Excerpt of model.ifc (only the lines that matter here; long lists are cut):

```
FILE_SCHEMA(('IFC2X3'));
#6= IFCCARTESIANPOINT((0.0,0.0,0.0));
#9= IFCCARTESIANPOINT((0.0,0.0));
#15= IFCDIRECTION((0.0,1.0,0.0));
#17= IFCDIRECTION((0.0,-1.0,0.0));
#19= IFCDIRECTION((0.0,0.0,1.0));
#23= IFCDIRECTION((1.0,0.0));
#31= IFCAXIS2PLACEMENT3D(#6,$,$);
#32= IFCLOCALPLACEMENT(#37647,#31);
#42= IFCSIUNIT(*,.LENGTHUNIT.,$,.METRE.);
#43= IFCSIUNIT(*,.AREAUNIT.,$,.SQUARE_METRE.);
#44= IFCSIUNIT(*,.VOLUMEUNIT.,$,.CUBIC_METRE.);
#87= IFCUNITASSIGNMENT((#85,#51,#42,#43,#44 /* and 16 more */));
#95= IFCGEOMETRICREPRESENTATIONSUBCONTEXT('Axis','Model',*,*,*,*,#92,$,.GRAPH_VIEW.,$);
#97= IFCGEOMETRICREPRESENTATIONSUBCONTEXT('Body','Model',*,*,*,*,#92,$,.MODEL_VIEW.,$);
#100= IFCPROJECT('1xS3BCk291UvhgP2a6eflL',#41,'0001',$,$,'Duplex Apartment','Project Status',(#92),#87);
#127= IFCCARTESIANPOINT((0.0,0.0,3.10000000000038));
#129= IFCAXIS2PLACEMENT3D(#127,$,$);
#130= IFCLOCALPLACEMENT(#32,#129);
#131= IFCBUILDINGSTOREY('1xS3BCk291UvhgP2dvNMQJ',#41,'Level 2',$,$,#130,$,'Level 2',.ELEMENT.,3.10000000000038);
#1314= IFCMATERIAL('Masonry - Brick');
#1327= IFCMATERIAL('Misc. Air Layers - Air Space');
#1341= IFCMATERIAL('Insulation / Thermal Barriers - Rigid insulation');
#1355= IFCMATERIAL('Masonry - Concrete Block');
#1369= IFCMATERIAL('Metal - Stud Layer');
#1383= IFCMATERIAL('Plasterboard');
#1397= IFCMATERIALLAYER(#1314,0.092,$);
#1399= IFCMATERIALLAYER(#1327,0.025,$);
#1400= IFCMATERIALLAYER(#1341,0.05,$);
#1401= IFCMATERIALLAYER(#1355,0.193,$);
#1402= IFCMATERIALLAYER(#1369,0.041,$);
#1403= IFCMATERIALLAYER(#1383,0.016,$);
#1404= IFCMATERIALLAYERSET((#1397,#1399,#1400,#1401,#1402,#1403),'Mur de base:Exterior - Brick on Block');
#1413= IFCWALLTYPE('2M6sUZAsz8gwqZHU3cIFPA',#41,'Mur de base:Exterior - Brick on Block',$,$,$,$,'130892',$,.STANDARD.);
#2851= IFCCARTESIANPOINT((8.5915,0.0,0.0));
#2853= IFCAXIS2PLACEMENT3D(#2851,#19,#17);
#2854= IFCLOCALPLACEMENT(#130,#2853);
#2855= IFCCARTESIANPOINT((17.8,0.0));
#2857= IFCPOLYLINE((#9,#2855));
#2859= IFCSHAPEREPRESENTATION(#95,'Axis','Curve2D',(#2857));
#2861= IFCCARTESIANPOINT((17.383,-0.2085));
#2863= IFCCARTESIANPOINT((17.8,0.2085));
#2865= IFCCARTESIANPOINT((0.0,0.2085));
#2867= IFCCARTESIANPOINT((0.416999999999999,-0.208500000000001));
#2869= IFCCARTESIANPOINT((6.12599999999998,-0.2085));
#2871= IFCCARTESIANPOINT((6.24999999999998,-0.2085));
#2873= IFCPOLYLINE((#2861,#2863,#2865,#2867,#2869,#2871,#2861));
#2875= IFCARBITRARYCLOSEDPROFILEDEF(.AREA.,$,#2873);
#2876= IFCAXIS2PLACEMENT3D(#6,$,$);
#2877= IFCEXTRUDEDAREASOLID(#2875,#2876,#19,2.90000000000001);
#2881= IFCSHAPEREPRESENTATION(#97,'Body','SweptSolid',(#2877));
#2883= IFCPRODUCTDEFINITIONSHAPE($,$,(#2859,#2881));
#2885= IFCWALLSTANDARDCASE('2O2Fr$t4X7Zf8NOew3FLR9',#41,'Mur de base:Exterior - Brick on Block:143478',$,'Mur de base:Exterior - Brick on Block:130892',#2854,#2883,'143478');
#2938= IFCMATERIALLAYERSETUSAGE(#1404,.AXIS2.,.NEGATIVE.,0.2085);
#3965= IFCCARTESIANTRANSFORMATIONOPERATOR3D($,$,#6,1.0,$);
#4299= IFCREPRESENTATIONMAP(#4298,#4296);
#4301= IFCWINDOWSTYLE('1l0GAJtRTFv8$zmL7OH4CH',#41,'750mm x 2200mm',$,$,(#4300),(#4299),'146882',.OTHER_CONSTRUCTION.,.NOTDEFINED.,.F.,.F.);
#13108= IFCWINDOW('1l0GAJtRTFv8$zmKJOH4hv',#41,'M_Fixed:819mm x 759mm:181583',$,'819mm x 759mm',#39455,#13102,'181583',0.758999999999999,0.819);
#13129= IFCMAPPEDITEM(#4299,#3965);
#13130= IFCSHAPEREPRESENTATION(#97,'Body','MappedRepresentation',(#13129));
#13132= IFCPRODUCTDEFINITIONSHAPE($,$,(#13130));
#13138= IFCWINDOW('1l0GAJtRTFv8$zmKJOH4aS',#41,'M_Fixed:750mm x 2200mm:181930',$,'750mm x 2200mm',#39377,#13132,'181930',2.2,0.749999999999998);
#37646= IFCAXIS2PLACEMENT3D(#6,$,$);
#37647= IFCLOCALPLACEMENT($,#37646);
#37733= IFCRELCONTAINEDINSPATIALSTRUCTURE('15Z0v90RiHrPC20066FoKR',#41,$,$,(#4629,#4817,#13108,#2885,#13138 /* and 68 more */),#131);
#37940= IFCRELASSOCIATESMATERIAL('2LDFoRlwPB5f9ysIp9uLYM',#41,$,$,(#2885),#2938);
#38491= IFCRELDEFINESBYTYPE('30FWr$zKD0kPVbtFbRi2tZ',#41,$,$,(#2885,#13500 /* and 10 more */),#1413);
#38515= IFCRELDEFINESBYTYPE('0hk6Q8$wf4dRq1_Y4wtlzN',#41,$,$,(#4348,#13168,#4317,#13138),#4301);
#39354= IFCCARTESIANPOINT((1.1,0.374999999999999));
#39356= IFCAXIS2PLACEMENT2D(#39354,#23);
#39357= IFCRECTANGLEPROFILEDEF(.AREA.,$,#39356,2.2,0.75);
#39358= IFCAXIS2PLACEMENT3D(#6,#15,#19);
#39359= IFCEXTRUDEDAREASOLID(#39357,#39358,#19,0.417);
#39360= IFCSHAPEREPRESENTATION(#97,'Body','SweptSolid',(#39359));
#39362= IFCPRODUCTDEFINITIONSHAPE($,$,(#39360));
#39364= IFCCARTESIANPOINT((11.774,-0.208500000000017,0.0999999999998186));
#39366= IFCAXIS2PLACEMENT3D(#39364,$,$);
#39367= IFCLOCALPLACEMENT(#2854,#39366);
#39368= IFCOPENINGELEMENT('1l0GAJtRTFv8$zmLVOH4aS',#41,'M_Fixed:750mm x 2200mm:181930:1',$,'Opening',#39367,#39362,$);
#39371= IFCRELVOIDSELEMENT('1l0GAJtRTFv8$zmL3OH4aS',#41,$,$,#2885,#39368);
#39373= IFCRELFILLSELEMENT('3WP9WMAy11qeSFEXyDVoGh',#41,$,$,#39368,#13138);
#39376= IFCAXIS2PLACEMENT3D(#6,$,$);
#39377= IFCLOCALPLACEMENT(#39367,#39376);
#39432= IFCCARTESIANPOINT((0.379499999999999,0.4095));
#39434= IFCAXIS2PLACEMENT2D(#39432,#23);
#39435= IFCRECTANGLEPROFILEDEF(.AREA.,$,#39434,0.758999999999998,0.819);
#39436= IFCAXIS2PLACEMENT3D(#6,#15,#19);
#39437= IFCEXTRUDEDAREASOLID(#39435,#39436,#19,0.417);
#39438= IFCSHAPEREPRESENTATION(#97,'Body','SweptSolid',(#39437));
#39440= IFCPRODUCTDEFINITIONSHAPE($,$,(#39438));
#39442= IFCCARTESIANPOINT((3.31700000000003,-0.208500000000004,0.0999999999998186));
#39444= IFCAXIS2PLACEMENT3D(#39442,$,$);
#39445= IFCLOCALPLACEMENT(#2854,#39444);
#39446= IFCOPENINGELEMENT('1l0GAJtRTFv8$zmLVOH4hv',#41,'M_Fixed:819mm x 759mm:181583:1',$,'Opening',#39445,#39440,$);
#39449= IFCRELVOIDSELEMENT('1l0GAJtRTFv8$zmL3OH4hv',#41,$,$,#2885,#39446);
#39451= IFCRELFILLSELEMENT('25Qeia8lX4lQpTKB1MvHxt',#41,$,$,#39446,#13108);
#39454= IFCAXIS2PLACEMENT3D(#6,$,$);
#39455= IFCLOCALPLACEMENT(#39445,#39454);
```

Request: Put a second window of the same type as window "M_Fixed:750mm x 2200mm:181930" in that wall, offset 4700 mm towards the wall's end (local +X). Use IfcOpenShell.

```python
import ifcopenshell
import ifcopenshell.api.feature
import ifcopenshell.api.geometry
import ifcopenshell.api.root
import ifcopenshell.geom
import ifcopenshell.util.element
import ifcopenshell.util.placement
import ifcopenshell.util.shape
import ifcopenshell.util.unit

model = ifcopenshell.open("model.ifc")
unit_scale = ifcopenshell.util.unit.calculate_unit_scale(model)
settings = ifcopenshell.geom.settings()


def volume(element):
    """Net volume in cubic metres, openings subtracted."""
    shape = ifcopenshell.geom.create_shape(settings, element)
    return ifcopenshell.util.shape.get_volume(shape.geometry)


def reuse_history(source, copy):
    """copy_class also copies each property set's owner history, people and application; keep the originals."""
    for rel in copy.IsDefinedBy:
        if rel.is_a("IfcRelDefinesByProperties") and (history := rel.RelatingPropertyDefinition.OwnerHistory):
            rel.RelatingPropertyDefinition.OwnerHistory = source.OwnerHistory
            ifcopenshell.util.element.remove_deep2(model, history)


window = model.by_guid("1l0GAJtRTFv8$zmKJOH4aS")
opening = window.FillsVoids[0].RelatingOpeningElement
wall = opening.VoidsElements[0].RelatingBuildingElement
before = volume(wall)
shift = ifcopenshell.util.placement.get_local_placement(wall.ObjectPlacement)[:3, 0] * 4.7 / unit_scale

# copy_class copies the void relationship, type, container and properties, but no geometry.
new_opening = ifcopenshell.api.root.copy_class(model, product=opening)
new_opening.Representation = ifcopenshell.util.element.copy_deep(
    model, opening.Representation, exclude=["IfcGeometricRepresentationContext", "IfcRepresentationMap"]
)
new_opening.Name = "M_Fixed:750mm x 2200mm"
new_window = ifcopenshell.api.root.copy_class(model, product=window)
new_window.Representation = ifcopenshell.util.element.copy_deep(
    model, window.Representation, exclude=["IfcGeometricRepresentationContext", "IfcRepresentationMap"]
)
new_window.Name = "M_Fixed:750mm x 2200mm"
new_window.Tag = None
reuse_history(window, new_window)
fills = ifcopenshell.api.feature.add_filling(model, opening=new_opening, element=new_window)
fills.OwnerHistory = new_window.OwnerHistory  # required in IFC2X3

for old, new in ((opening, new_opening), (window, new_window)):
    matrix = ifcopenshell.util.placement.get_local_placement(old.ObjectPlacement)
    matrix[:3, 3] += shift
    ifcopenshell.api.geometry.edit_object_placement(model, product=new, matrix=matrix, is_si=False)

after = volume(wall)

print(f"wall volume {before:.3f} -> {after:.3f} m3")

model.write("model_v2.ifc")
```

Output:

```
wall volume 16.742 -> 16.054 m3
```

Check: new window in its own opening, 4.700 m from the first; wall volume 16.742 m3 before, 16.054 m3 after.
